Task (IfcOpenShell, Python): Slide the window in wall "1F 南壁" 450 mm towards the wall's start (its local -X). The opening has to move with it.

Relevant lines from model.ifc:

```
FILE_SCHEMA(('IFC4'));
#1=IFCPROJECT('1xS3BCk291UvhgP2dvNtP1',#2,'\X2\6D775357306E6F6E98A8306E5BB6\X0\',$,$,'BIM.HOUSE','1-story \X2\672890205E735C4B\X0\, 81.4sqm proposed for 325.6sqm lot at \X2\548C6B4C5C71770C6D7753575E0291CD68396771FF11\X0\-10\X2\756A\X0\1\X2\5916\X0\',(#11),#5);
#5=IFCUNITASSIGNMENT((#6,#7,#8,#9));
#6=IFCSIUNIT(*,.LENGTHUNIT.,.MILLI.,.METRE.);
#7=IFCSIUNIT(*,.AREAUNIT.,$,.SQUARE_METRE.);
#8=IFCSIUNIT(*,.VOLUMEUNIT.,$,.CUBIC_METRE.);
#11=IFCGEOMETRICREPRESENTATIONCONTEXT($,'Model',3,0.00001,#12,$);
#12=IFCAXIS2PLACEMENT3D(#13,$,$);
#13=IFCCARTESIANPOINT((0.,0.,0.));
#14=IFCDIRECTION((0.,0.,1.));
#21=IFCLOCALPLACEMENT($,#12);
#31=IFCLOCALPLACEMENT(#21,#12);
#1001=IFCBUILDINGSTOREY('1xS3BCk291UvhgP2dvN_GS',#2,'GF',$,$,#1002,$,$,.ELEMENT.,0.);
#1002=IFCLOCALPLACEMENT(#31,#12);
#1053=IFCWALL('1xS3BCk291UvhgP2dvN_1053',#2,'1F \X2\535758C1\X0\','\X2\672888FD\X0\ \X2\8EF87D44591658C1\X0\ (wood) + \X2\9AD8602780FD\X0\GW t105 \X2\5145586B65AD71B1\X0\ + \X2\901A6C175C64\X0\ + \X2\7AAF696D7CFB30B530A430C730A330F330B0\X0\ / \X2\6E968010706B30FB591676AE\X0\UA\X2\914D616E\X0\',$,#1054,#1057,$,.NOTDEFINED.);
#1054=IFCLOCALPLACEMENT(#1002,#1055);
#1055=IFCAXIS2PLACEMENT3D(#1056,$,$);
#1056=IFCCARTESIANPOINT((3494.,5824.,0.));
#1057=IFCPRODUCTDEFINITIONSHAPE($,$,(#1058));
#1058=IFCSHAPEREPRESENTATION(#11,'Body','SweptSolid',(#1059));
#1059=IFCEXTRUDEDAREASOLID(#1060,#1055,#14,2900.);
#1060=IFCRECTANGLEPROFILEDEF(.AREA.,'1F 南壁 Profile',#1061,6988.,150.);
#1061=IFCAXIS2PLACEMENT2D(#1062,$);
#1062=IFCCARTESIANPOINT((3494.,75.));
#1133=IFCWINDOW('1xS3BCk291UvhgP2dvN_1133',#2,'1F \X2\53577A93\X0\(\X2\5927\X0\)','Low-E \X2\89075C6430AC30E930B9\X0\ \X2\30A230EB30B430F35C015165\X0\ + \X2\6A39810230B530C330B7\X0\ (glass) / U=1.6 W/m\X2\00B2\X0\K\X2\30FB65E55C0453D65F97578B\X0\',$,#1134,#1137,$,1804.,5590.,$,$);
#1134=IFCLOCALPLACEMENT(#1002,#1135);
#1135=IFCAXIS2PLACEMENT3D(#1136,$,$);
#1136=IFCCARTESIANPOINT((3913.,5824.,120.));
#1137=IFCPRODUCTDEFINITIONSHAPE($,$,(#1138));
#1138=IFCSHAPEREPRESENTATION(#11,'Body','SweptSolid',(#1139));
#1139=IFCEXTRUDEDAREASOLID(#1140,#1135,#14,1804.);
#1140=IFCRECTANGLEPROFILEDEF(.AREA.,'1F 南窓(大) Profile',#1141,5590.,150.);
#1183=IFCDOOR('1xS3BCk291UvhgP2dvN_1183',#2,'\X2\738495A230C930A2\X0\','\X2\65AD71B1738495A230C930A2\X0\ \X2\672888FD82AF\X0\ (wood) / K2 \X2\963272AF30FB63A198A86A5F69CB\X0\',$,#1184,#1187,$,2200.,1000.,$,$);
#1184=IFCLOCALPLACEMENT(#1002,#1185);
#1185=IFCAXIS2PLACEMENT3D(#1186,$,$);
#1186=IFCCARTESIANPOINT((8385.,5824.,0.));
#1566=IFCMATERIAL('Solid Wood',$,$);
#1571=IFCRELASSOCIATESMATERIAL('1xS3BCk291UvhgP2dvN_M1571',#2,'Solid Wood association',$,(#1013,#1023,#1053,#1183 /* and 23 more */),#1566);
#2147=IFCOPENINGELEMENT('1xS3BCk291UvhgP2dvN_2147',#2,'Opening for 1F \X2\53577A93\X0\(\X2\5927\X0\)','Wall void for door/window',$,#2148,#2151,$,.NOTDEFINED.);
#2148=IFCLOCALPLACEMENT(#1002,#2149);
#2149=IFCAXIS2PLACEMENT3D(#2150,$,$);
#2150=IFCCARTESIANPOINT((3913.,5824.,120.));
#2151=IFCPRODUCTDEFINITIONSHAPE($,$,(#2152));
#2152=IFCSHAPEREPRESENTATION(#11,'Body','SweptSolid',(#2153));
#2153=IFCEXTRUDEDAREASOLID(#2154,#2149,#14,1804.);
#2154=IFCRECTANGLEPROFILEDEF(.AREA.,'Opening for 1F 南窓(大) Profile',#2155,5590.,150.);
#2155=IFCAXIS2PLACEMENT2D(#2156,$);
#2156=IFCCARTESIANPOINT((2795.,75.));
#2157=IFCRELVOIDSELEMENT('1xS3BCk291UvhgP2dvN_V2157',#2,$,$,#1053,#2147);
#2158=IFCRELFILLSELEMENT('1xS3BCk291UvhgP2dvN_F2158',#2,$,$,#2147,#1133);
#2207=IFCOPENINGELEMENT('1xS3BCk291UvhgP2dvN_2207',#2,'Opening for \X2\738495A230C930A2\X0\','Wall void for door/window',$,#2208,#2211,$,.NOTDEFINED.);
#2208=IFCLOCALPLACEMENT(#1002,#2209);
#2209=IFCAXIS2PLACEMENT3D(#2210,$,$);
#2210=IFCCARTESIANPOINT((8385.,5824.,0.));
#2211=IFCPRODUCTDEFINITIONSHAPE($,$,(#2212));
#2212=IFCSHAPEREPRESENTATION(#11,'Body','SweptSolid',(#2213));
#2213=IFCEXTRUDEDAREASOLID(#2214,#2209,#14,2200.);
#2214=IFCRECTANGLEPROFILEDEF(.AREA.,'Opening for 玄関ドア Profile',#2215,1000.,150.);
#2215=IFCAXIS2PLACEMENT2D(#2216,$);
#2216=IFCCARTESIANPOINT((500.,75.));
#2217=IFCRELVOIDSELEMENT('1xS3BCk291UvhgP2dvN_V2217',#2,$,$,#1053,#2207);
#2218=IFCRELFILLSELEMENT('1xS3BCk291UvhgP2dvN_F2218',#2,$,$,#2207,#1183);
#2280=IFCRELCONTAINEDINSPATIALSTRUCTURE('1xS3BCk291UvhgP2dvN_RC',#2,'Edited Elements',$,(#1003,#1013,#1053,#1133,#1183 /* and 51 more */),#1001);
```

```python
import ifcopenshell
import ifcopenshell.api.geometry
import ifcopenshell.util.placement
import ifcopenshell.util.unit

model = ifcopenshell.open("model.ifc")
unit_scale = ifcopenshell.util.unit.calculate_unit_scale(model)

window = model.by_guid("1xS3BCk291UvhgP2dvN_1133")
opening = window.FillsVoids[0].RelatingOpeningElement
wall = opening.VoidsElements[0].RelatingBuildingElement

wall_matrix = ifcopenshell.util.placement.get_local_placement(wall.ObjectPlacement)
shift = wall_matrix[:3, 0] * -0.45 / unit_scale
before = ifcopenshell.util.placement.get_local_placement(window.ObjectPlacement)[:3, 3].copy()

# The window is not placed relative to its opening, so move both.
for product in (opening, window):
    matrix = ifcopenshell.util.placement.get_local_placement(product.ObjectPlacement)
    matrix[:3, 3] += shift
    ifcopenshell.api.geometry.edit_object_placement(model, product=product, matrix=matrix, is_si=False)

after = ifcopenshell.util.placement.get_local_placement(window.ObjectPlacement)[:3, 3]
print("window moved by", (after - before).round(3) + 0.0)

model.write("model_updated.ifc")
```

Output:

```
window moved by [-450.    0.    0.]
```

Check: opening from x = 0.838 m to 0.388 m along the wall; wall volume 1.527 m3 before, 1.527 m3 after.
